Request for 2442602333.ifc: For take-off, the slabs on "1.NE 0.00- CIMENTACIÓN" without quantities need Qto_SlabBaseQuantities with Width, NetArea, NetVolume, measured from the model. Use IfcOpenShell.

First a look at what the model holds.

```python
import ifcopenshell
import ifcopenshell.util.element
import ifcopenshell.util.unit

model = ifcopenshell.open("2442602333.ifc")
print(model.schema)
for unit_type in ("LENGTHUNIT", "AREAUNIT", "VOLUMEUNIT"):
    print(unit_type, ifcopenshell.util.unit.calculate_unit_scale(model, unit_type))
storey = next(s for s in model.by_type("IfcBuildingStorey") if s.Name == "1.NE 0.00- CIMENTACIÓN")
slabs = [e for e in ifcopenshell.util.element.get_decomposition(storey) if e.is_a("IfcSlab")]
for e in sorted(slabs, key=lambda e: e.id()):
    print(e.id(), e.is_a(), e.Name, list(ifcopenshell.util.element.get_psets(e, qtos_only=True)), sep=" | ")
```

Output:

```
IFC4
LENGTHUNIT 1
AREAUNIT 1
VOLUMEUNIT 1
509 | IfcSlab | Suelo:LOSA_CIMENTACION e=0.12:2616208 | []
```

```python
import ifcopenshell
import ifcopenshell.api.pset
import ifcopenshell.geom
import ifcopenshell.util.element
import ifcopenshell.util.shape
import ifcopenshell.util.unit

model = ifcopenshell.open("2442602333.ifc")
unit_scale = ifcopenshell.util.unit.calculate_unit_scale(model)
area_scale = ifcopenshell.util.unit.calculate_unit_scale(model, "AREAUNIT")
volume_scale = ifcopenshell.util.unit.calculate_unit_scale(model, "VOLUMEUNIT")
settings = ifcopenshell.geom.settings()

storey = next(s for s in model.by_type("IfcBuildingStorey") if s.Name == "1.NE 0.00- CIMENTACIÓN")
slabs = [e for e in ifcopenshell.util.element.get_decomposition(storey) if e.is_a("IfcSlab")]

for e in sorted(slabs, key=lambda e: e.id()):
    if ifcopenshell.util.element.get_psets(e, qtos_only=True, should_inherit=False):
        continue
    # Geometry comes back in metres, in the element's own axes.
    shape = ifcopenshell.geom.create_shape(settings, e)
    values = {
        "Width": ifcopenshell.util.shape.get_z(shape.geometry) / unit_scale,
        "NetArea": ifcopenshell.util.shape.get_footprint_area(shape.geometry) / area_scale,
        "NetVolume": ifcopenshell.util.shape.get_volume(shape.geometry) / volume_scale,
    }
    qto = ifcopenshell.api.pset.add_qto(model, product=e, name="Qto_SlabBaseQuantities")
    ifcopenshell.api.pset.edit_qto(model, qto=qto, properties=values)
    print(e.id(), {k: round(v, 3) for k, v in values.items()})

model.write("2442602333_edited.ifc")
```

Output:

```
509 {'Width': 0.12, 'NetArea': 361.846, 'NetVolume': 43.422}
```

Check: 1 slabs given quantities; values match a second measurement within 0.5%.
